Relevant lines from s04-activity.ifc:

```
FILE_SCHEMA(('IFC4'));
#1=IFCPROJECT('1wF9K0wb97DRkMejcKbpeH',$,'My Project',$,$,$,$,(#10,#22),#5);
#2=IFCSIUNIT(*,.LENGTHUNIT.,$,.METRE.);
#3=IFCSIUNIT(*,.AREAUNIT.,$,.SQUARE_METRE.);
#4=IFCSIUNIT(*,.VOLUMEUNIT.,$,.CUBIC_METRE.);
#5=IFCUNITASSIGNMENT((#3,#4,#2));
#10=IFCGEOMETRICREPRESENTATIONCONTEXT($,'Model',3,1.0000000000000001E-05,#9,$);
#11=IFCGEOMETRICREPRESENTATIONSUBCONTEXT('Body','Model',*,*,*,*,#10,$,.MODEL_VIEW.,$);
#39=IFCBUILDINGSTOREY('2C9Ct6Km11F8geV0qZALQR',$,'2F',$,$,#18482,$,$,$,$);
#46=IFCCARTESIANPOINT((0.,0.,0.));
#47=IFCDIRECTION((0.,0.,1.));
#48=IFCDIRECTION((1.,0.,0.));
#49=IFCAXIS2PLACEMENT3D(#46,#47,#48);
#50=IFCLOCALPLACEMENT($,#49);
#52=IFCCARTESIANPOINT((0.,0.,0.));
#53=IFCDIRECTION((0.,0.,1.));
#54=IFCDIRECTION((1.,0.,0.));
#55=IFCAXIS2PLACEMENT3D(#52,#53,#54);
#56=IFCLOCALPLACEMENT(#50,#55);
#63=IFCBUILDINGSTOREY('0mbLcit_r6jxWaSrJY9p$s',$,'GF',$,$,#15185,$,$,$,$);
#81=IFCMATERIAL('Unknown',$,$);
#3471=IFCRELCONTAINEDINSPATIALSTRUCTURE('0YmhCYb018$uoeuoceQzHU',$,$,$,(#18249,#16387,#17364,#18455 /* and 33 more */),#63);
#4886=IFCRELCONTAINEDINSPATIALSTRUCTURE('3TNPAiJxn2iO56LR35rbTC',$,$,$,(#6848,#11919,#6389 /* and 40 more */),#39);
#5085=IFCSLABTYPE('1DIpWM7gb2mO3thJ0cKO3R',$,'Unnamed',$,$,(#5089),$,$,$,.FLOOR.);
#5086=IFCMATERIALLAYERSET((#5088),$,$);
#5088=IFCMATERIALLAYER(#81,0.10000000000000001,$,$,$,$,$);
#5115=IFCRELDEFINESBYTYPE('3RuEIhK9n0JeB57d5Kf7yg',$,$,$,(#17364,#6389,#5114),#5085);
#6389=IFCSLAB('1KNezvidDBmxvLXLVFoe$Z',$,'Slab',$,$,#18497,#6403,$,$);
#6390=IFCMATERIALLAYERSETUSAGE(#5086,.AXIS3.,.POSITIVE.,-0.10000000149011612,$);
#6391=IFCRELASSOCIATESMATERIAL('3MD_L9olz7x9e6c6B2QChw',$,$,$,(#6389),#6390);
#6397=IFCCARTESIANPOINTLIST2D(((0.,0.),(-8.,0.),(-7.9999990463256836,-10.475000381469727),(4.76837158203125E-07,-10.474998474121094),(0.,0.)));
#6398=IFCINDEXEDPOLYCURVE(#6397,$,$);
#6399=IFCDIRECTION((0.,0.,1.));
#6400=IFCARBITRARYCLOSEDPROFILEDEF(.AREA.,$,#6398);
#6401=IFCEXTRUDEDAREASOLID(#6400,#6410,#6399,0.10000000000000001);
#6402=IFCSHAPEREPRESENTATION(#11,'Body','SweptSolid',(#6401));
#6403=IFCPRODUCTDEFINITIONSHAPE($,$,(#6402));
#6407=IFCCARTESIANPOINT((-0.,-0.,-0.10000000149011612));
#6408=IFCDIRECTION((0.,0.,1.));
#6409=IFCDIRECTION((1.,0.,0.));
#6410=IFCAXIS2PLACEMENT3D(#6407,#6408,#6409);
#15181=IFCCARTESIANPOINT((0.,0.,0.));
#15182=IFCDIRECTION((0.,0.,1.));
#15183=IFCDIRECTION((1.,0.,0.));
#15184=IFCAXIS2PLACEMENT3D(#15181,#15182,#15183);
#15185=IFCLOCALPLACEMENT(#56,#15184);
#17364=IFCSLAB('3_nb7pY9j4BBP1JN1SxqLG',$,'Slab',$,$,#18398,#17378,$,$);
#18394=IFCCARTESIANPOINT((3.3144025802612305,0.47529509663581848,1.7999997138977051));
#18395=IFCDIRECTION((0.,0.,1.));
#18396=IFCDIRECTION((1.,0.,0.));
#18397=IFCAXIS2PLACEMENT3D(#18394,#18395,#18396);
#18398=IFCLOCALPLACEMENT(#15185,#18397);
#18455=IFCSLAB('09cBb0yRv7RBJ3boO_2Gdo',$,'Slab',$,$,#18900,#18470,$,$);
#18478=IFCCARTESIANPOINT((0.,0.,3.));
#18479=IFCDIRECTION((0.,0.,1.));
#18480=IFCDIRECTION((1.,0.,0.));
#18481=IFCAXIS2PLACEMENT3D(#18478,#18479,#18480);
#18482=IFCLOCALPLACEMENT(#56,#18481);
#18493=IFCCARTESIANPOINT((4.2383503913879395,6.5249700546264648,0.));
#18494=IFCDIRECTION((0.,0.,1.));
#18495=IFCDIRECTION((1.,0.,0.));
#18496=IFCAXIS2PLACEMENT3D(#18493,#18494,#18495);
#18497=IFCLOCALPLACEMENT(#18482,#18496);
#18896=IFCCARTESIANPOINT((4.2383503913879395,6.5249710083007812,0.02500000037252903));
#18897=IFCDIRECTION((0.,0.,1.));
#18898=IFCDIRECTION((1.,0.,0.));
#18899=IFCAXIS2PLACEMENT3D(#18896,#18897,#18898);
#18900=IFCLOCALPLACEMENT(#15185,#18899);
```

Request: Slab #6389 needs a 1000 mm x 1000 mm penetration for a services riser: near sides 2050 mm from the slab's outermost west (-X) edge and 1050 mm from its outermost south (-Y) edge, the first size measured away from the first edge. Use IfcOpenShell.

```python
import numpy as np
import ifcopenshell
import ifcopenshell.api.feature
import ifcopenshell.api.geometry
import ifcopenshell.api.root
import ifcopenshell.geom
import ifcopenshell.util.placement
import ifcopenshell.util.representation
import ifcopenshell.util.shape
import ifcopenshell.util.unit

model = ifcopenshell.open("s04-activity.ifc")
unit_scale = ifcopenshell.util.unit.calculate_unit_scale(model)
settings = ifcopenshell.geom.settings()


def volume(element):
    """Net volume in cubic metres, openings subtracted."""
    shape = ifcopenshell.geom.create_shape(settings, element)
    return ifcopenshell.util.shape.get_volume(shape.geometry)


slab = model.by_id(6389)
before = volume(slab)

# Extent in the slab's own axes, in metres. The edges named are its -X and -Y sides.
slab_shape = ifcopenshell.geom.create_shape(settings, slab)
vertices = ifcopenshell.util.shape.get_vertices(slab_shape.geometry)
x_min, y_min, bottom = vertices.min(axis=0)
top = vertices[:, 2].max()

opening = ifcopenshell.api.root.create_entity(model, ifc_class="IfcOpeningElement", name="Services riser opening", predefined_type="OPENING")
context = ifcopenshell.util.representation.get_context(model, "Model", "Body", "MODEL_VIEW")
width, depth = 1, 1
outline = [(0.0, 0.0), (width, 0.0), (width, depth), (0.0, depth), (0.0, 0.0)]
# Overshoot both faces by 50 mm so the cut is clean.
shape = ifcopenshell.api.geometry.add_slab_representation(
    model, context=context, depth=top - bottom + 0.1, polyline=outline
)
ifcopenshell.api.geometry.assign_representation(model, product=opening, representation=shape)

matrix = ifcopenshell.util.placement.get_local_placement(slab.ObjectPlacement)
matrix[:, 3] = matrix @ np.append(np.array([x_min + 2.05, y_min + 1.05, bottom - 0.05]) / unit_scale, 1.0)
ifcopenshell.api.geometry.edit_object_placement(model, product=opening, matrix=matrix, is_si=False)
ifcopenshell.api.feature.add_feature(model, feature=opening, element=slab)

after = volume(slab)

print(f"slab volume {before:.3f} -> {after:.3f} m3")

model.write("s04-activity_updated.ifc")
```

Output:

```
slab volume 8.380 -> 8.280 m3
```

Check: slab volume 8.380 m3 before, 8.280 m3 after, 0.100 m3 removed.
